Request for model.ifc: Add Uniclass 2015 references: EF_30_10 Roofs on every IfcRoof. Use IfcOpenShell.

First a look at what the model holds.

```python
import ifcopenshell

model = ifcopenshell.open("model.ifc")
print(model.schema)
print("classifications:", [c.Name for c in model.by_type("IfcClassification")])
for ifc_class in ("IfcDoor", "IfcRoof", "IfcStair", "IfcWall", "IfcWindow"):
    print(ifc_class, len(model.by_type(ifc_class)))
```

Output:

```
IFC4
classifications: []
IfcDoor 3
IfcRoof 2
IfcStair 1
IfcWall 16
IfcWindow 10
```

```python
import ifcopenshell
import ifcopenshell.api.classification

model = ifcopenshell.open("model.ifc")

system = ifcopenshell.api.classification.add_classification(model, classification="Uniclass 2015")

codes = {
    "IfcRoof": ("EF_30_10", "Roofs"),
}
for ifc_class, (code, name) in codes.items():
    products = model.by_type(ifc_class)
    ifcopenshell.api.classification.add_reference(
        model, products=products, classification=system, identification=code, name=name
    )
    print(code, len(products))

model.write("model-out.ifc")
```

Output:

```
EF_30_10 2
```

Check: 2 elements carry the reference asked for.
